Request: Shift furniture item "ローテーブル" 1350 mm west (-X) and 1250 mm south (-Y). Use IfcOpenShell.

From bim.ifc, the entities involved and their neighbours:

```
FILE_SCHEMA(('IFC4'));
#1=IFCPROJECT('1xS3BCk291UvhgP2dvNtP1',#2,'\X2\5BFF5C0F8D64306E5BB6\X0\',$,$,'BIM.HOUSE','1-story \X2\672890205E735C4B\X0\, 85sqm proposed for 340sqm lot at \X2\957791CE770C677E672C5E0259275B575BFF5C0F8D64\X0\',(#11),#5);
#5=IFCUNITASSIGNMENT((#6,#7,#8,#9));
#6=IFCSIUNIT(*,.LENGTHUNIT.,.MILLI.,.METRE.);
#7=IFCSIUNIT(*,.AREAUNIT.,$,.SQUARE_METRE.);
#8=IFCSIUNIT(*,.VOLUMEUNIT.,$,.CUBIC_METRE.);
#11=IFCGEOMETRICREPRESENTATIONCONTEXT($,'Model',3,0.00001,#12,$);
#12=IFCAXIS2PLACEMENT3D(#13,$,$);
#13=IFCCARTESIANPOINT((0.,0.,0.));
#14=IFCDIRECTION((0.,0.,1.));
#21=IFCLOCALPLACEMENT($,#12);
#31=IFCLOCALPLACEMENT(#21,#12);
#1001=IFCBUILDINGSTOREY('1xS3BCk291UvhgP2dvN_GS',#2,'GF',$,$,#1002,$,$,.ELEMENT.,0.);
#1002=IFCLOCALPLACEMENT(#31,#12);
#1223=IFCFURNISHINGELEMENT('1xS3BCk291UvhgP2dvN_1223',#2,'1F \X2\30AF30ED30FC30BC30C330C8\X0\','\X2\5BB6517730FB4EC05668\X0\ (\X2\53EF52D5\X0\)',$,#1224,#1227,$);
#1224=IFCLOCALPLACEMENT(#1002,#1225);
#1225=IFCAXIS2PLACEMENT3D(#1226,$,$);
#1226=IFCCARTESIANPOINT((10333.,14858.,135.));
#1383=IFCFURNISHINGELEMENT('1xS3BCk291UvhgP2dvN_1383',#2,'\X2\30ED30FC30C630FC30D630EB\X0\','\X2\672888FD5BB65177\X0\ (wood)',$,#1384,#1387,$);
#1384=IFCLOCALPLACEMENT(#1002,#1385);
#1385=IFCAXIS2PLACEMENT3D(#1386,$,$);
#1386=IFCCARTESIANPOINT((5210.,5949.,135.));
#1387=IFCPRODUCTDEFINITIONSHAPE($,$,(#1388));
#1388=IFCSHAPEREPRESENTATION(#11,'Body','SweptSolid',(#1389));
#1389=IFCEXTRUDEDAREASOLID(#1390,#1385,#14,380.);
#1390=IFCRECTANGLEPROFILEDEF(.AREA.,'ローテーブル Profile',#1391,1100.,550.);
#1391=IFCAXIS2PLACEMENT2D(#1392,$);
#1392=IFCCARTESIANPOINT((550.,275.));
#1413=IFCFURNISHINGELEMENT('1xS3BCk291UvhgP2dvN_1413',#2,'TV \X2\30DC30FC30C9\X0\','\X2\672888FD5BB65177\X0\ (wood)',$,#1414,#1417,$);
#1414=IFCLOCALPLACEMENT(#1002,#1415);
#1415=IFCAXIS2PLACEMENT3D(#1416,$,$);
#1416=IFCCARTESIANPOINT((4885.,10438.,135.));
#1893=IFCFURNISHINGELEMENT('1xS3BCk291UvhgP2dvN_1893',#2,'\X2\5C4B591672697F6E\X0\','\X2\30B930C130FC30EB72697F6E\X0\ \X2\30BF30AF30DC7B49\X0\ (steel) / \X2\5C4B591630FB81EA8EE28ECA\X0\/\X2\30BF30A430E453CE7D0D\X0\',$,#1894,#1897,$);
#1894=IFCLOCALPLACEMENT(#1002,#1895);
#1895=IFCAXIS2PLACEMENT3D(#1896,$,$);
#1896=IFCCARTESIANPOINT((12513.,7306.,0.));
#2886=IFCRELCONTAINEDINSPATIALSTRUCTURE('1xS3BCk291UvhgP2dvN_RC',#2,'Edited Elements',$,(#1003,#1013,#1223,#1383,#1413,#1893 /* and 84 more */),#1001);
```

```python
import ifcopenshell
import ifcopenshell.api.geometry
import ifcopenshell.util.placement

model = ifcopenshell.open("bim.ifc")

item = model.by_guid("1xS3BCk291UvhgP2dvN_1383")
matrix = ifcopenshell.util.placement.get_local_placement(item.ObjectPlacement)
matrix[0, 3] -= 1350.0
matrix[1, 3] -= 1250.0
ifcopenshell.api.geometry.edit_object_placement(model, product=item, matrix=matrix, is_si=False)

print(ifcopenshell.util.placement.get_local_placement(item.ObjectPlacement).round(3) + 0.0)

model.write("bim_rev.ifc")
```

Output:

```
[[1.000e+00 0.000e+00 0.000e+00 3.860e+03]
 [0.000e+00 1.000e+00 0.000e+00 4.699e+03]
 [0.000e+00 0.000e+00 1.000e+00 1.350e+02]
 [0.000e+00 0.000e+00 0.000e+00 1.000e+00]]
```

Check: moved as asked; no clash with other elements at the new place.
